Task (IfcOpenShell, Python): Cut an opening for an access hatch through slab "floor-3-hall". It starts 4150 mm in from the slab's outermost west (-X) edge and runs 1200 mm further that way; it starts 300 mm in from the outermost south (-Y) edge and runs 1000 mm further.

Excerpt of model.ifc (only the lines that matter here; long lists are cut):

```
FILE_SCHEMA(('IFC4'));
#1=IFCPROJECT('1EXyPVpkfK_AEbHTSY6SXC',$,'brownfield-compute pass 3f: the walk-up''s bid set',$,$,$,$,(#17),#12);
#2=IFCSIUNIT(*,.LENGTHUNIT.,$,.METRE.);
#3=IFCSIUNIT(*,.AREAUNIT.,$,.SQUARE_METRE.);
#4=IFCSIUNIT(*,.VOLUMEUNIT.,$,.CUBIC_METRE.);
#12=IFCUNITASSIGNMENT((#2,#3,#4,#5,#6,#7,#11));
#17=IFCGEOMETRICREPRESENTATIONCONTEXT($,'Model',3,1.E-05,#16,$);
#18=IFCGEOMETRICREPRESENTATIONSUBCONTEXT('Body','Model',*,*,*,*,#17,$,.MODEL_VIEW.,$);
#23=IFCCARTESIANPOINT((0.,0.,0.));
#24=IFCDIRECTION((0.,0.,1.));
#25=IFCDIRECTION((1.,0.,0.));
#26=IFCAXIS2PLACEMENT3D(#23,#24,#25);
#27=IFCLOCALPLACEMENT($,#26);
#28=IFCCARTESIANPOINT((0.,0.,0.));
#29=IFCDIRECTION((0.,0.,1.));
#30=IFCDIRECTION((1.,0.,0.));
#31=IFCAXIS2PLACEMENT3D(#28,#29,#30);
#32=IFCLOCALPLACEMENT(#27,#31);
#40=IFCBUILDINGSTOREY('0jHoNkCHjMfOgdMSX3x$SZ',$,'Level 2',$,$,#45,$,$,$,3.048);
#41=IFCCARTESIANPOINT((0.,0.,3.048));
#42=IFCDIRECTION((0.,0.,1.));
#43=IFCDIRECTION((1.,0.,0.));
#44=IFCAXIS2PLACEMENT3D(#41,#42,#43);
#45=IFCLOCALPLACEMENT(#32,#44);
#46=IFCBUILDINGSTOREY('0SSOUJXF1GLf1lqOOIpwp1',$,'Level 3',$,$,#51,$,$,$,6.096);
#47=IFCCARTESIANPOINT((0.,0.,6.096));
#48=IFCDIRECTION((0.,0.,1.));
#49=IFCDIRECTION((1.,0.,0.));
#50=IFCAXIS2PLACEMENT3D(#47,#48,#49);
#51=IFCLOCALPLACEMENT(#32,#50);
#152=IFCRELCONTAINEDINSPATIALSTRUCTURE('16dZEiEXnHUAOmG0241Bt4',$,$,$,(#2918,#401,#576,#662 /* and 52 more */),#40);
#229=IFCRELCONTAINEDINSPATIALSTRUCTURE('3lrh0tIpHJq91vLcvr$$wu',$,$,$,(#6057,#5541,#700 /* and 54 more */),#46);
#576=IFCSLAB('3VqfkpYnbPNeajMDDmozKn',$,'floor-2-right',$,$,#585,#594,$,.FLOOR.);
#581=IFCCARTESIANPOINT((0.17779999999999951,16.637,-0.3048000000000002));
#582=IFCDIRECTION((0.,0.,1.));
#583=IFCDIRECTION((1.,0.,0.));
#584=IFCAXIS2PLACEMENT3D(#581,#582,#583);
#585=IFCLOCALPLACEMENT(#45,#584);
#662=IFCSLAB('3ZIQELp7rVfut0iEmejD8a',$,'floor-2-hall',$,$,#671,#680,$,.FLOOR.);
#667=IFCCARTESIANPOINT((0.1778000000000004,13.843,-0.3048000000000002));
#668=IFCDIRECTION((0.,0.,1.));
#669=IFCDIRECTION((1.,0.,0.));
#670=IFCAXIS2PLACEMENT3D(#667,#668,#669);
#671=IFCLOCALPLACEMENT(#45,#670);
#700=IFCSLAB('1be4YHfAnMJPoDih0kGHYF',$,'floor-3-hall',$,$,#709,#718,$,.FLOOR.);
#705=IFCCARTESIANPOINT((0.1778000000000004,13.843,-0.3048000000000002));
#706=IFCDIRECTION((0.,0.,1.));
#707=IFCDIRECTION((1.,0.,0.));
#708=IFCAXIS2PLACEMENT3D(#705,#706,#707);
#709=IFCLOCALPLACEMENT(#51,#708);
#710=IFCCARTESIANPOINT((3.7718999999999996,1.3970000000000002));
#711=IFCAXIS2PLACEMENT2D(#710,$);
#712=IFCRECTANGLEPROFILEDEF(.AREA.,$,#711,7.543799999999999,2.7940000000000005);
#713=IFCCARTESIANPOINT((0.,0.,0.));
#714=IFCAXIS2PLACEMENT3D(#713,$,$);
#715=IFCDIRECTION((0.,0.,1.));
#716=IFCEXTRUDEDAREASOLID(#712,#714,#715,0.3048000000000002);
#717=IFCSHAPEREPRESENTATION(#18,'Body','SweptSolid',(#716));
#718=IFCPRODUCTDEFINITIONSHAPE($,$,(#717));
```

```python
import numpy as np
import ifcopenshell
import ifcopenshell.api.feature
import ifcopenshell.api.geometry
import ifcopenshell.api.root
import ifcopenshell.geom
import ifcopenshell.util.placement
import ifcopenshell.util.representation
import ifcopenshell.util.shape
import ifcopenshell.util.unit

model = ifcopenshell.open("model.ifc")
unit_scale = ifcopenshell.util.unit.calculate_unit_scale(model)
settings = ifcopenshell.geom.settings()


def volume(element):
    """Net volume in cubic metres, openings subtracted."""
    shape = ifcopenshell.geom.create_shape(settings, element)
    return ifcopenshell.util.shape.get_volume(shape.geometry)


slab = model.by_guid("1be4YHfAnMJPoDih0kGHYF")
before = volume(slab)

# Extent in the slab's own axes, in metres. The edges named are its -X and -Y sides.
slab_shape = ifcopenshell.geom.create_shape(settings, slab)
vertices = ifcopenshell.util.shape.get_vertices(slab_shape.geometry)
x_min, y_min, bottom = vertices.min(axis=0)
top = vertices[:, 2].max()

opening = ifcopenshell.api.root.create_entity(model, ifc_class="IfcOpeningElement", name="Access hatch opening", predefined_type="OPENING")
context = ifcopenshell.util.representation.get_context(model, "Model", "Body", "MODEL_VIEW")
width, depth = 1.2, 1
outline = [(0.0, 0.0), (width, 0.0), (width, depth), (0.0, depth), (0.0, 0.0)]
# Overshoot both faces by 50 mm so the cut is clean.
shape = ifcopenshell.api.geometry.add_slab_representation(
    model, context=context, depth=top - bottom + 0.1, polyline=outline
)
ifcopenshell.api.geometry.assign_representation(model, product=opening, representation=shape)

matrix = ifcopenshell.util.placement.get_local_placement(slab.ObjectPlacement)
matrix[:, 3] = matrix @ np.append(np.array([x_min + 4.15, y_min + 0.3, bottom - 0.05]) / unit_scale, 1.0)
ifcopenshell.api.geometry.edit_object_placement(model, product=opening, matrix=matrix, is_si=False)
ifcopenshell.api.feature.add_feature(model, feature=opening, element=slab)

after = volume(slab)

print(f"slab volume {before:.3f} -> {after:.3f} m3")

model.write("model-out.ifc")
```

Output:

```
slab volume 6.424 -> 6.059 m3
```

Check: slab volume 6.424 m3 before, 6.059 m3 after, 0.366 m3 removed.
